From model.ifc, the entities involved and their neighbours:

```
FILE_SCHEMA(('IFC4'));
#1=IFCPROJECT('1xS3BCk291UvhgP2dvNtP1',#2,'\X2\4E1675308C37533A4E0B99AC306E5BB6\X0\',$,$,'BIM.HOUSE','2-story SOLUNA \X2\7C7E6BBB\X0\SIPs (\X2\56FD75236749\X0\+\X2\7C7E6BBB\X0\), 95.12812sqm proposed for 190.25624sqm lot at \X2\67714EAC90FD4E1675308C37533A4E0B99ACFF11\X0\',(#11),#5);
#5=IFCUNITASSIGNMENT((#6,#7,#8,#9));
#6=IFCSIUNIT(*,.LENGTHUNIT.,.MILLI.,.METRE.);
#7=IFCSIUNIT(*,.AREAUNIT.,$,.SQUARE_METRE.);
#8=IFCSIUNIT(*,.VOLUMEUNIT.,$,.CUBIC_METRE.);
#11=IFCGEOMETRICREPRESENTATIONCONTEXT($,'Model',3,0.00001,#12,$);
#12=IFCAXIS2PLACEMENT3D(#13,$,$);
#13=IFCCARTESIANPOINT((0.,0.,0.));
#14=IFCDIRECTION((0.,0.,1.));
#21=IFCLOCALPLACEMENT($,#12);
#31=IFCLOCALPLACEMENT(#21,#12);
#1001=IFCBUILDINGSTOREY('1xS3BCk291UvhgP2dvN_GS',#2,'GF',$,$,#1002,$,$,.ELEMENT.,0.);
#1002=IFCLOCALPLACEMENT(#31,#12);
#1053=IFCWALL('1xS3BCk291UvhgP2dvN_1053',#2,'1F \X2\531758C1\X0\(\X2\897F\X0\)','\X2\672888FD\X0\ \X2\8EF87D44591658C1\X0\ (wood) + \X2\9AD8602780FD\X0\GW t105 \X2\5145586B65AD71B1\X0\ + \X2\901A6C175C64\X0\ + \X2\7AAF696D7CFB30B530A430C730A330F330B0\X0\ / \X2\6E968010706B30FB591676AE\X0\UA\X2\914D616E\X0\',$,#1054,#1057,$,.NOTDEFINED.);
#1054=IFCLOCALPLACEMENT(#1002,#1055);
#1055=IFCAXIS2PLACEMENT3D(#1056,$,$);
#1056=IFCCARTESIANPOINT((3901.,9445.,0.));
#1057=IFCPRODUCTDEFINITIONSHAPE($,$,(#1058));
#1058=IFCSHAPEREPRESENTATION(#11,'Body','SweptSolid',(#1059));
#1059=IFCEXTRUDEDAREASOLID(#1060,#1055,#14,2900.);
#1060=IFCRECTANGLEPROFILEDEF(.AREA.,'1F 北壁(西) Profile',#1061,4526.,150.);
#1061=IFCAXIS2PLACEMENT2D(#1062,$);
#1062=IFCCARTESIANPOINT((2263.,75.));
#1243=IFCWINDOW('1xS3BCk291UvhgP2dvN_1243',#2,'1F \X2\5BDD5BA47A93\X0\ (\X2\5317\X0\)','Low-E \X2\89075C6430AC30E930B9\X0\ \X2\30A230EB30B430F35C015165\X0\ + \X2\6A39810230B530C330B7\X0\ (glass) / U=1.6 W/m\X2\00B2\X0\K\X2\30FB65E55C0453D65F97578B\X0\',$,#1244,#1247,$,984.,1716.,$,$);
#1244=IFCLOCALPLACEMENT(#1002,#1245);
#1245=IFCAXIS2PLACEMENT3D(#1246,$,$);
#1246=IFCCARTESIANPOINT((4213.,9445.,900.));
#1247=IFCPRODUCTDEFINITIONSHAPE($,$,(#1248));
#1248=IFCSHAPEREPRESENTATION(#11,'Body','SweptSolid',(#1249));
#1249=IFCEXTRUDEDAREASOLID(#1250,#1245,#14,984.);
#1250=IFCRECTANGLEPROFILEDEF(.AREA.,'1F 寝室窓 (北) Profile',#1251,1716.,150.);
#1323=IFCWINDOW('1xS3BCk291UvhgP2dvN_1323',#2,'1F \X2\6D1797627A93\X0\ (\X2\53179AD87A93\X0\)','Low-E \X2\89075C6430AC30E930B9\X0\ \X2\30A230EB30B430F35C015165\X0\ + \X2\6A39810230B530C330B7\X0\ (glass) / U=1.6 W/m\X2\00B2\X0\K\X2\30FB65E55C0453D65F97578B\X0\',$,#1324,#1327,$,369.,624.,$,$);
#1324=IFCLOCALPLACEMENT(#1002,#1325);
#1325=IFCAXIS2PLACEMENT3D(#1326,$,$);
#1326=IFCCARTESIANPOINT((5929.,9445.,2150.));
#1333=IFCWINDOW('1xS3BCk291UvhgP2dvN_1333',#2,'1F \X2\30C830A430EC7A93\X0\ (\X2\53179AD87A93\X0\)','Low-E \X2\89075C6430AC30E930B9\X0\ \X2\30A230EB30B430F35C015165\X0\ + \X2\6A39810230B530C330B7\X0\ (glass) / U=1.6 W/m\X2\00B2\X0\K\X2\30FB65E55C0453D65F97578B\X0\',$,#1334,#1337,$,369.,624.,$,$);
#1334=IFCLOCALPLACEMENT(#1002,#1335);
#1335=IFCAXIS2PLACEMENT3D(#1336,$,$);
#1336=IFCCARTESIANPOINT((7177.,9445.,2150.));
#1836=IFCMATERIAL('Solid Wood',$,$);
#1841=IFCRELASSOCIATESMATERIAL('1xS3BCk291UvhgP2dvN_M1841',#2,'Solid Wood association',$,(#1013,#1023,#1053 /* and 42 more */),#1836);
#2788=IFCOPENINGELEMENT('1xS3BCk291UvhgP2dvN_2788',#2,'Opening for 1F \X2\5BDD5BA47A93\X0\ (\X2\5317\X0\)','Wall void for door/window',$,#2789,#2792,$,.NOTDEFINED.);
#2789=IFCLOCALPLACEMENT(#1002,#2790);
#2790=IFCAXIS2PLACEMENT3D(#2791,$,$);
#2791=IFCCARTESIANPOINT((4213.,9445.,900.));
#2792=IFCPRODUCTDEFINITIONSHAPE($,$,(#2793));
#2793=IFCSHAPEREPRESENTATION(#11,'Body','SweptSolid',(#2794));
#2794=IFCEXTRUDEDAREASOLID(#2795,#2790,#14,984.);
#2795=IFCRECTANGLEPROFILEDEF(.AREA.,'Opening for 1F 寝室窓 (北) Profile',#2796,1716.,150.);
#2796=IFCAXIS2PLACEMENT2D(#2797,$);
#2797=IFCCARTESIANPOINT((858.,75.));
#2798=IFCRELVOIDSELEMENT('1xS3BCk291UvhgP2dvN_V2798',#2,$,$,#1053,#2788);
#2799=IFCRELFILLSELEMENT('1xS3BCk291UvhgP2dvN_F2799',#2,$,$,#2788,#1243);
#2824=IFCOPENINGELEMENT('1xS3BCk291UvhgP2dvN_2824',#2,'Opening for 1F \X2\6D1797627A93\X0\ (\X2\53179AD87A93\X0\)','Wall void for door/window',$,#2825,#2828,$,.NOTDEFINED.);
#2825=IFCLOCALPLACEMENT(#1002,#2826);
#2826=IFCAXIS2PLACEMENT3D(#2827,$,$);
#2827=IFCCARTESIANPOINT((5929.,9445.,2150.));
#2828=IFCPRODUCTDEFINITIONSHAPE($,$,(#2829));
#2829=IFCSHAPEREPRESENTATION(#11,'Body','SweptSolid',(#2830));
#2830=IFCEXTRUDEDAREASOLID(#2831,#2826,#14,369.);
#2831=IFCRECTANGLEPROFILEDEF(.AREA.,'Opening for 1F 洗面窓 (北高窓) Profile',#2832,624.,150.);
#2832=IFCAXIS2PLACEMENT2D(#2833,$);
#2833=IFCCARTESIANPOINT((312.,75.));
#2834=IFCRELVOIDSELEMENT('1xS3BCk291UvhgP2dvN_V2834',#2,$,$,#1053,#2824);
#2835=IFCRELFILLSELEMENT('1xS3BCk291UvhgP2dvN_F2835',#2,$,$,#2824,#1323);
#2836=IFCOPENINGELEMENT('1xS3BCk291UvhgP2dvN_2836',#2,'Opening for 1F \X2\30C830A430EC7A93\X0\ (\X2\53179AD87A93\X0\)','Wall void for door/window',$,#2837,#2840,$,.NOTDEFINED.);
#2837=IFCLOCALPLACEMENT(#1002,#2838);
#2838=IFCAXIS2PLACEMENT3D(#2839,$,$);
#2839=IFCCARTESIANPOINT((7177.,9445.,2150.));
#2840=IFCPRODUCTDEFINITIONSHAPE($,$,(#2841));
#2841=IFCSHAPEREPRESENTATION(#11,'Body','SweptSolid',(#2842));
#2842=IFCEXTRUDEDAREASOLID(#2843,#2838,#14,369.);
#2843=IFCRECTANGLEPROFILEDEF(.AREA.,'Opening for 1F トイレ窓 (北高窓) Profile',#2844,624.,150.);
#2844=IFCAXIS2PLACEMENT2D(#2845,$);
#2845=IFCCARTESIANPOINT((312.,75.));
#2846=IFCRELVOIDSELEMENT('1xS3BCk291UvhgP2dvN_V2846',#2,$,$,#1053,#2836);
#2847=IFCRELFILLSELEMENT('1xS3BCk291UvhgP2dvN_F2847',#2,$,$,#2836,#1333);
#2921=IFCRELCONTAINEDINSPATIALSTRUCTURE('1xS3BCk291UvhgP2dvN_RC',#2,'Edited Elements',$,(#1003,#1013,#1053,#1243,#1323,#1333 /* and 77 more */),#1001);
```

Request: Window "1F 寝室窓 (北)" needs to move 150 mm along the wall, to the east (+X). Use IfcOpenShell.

```python
import ifcopenshell
import ifcopenshell.api.geometry
import ifcopenshell.util.placement

model = ifcopenshell.open("model.ifc")

window = model.by_guid("1xS3BCk291UvhgP2dvN_1243")
opening = window.FillsVoids[0].RelatingOpeningElement
wall = opening.VoidsElements[0].RelatingBuildingElement

wall_matrix = ifcopenshell.util.placement.get_local_placement(wall.ObjectPlacement)
shift = wall_matrix[:3, 0] * 150.0
before = ifcopenshell.util.placement.get_local_placement(window.ObjectPlacement)[:3, 3].copy()

# The window is not placed relative to its opening, so move both.
for product in (opening, window):
    matrix = ifcopenshell.util.placement.get_local_placement(product.ObjectPlacement)
    matrix[:3, 3] += shift
    ifcopenshell.api.geometry.edit_object_placement(model, product=product, matrix=matrix, is_si=False)

after = ifcopenshell.util.placement.get_local_placement(window.ObjectPlacement)[:3, 3]
print("window moved by", (after - before).round(3) + 0.0)

model.write("model_edited.ifc")
```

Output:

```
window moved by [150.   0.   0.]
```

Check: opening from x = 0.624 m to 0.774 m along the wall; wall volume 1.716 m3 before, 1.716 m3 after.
